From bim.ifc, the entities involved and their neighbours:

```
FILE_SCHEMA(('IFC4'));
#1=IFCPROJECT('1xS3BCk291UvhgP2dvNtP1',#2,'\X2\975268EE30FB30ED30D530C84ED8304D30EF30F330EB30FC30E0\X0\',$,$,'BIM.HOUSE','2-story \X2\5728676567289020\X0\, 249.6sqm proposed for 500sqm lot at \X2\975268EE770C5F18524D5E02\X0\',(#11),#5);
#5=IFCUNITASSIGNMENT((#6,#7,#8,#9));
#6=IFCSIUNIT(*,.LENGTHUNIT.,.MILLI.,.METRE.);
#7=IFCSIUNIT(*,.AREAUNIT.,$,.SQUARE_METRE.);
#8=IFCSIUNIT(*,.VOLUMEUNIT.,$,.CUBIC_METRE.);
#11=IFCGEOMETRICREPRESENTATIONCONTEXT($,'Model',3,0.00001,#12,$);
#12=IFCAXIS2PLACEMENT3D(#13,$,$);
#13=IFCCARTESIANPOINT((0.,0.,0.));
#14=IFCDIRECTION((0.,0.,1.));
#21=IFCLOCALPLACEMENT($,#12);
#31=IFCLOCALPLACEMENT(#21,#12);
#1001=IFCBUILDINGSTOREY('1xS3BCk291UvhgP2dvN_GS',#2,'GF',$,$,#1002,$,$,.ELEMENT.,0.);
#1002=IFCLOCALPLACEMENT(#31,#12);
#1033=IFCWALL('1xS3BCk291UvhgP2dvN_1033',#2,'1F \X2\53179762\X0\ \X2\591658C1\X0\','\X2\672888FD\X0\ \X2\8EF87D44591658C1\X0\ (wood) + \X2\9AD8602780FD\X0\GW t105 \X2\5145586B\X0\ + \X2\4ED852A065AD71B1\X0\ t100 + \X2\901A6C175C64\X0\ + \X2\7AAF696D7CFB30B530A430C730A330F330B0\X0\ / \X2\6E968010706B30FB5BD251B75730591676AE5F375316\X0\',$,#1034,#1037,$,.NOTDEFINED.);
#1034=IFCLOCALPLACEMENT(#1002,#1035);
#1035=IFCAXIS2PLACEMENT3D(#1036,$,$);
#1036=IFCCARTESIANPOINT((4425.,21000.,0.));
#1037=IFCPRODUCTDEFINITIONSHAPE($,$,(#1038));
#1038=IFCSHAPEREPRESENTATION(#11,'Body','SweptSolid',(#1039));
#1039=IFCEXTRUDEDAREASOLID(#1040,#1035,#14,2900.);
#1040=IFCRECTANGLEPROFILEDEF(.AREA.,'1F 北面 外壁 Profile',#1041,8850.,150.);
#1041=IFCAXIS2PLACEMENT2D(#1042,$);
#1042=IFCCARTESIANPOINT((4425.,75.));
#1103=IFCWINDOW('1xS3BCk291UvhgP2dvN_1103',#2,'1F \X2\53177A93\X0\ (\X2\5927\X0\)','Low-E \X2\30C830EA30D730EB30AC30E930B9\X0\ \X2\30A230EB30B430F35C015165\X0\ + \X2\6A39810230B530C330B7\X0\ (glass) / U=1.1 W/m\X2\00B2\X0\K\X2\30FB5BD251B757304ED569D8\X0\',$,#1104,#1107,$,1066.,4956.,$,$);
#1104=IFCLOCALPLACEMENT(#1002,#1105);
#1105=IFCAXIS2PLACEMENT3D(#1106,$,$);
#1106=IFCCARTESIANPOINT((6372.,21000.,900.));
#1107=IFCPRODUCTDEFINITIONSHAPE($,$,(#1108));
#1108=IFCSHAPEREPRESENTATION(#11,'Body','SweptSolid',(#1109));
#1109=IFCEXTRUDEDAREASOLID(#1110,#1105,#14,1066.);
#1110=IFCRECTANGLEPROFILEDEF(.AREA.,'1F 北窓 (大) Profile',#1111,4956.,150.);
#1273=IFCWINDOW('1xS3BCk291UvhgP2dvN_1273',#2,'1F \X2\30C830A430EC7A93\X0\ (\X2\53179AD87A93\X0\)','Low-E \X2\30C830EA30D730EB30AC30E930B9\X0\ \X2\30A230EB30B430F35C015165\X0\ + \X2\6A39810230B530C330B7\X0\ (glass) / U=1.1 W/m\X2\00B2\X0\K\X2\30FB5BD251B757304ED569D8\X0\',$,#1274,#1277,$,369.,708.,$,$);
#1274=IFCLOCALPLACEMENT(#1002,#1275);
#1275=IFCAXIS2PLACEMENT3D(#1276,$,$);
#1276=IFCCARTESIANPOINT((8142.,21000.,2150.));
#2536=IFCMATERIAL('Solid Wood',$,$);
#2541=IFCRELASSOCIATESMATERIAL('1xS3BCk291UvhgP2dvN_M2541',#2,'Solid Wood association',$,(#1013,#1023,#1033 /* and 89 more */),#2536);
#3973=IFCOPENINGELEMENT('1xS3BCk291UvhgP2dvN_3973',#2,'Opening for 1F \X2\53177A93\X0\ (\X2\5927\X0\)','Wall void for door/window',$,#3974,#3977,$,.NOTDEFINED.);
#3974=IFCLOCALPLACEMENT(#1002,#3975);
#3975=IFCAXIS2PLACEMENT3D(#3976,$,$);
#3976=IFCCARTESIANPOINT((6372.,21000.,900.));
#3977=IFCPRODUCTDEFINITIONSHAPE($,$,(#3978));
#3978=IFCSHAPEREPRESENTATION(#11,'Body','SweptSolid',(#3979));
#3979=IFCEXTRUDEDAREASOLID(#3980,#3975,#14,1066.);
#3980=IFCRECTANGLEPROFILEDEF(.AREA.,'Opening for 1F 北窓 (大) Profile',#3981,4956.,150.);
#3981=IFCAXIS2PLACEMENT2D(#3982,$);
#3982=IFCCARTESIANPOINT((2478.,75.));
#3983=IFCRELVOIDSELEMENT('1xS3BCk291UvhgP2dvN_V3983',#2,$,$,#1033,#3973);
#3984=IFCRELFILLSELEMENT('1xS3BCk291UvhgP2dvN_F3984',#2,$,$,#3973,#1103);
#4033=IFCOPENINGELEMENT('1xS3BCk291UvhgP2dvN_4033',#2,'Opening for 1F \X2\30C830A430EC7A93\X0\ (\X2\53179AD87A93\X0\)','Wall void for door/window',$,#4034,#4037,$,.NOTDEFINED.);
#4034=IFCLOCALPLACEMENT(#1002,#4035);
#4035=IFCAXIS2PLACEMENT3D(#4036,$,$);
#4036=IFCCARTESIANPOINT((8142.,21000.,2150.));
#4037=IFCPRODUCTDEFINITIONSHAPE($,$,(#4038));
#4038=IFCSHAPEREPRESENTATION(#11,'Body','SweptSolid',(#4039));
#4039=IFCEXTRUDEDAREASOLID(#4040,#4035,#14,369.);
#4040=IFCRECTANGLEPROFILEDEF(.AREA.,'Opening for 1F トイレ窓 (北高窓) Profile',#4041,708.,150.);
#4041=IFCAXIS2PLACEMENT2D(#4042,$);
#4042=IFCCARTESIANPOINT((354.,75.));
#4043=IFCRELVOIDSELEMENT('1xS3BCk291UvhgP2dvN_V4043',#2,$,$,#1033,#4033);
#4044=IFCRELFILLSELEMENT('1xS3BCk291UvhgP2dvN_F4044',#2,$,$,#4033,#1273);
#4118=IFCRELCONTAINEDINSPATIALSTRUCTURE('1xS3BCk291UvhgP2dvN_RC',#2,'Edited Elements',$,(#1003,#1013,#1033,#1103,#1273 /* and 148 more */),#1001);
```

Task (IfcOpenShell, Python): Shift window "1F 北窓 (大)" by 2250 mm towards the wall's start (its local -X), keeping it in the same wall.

```python
import ifcopenshell
import ifcopenshell.api.geometry
import ifcopenshell.util.placement
import ifcopenshell.util.unit

model = ifcopenshell.open("bim.ifc")
unit_scale = ifcopenshell.util.unit.calculate_unit_scale(model)

window = model.by_guid("1xS3BCk291UvhgP2dvN_1103")
opening = window.FillsVoids[0].RelatingOpeningElement
wall = opening.VoidsElements[0].RelatingBuildingElement

wall_matrix = ifcopenshell.util.placement.get_local_placement(wall.ObjectPlacement)
shift = wall_matrix[:3, 0] * -2.25 / unit_scale
before = ifcopenshell.util.placement.get_local_placement(window.ObjectPlacement)[:3, 3].copy()

# The window is not placed relative to its opening, so move both.
for product in (opening, window):
    matrix = ifcopenshell.util.placement.get_local_placement(product.ObjectPlacement)
    matrix[:3, 3] += shift
    ifcopenshell.api.geometry.edit_object_placement(model, product=product, matrix=matrix, is_si=False)

after = ifcopenshell.util.placement.get_local_placement(window.ObjectPlacement)[:3, 3]
print("window moved by", (after - before).round(3) + 0.0)

model.write("bim_v2.ifc")
```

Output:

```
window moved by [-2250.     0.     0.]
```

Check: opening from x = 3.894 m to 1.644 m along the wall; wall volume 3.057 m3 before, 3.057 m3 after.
